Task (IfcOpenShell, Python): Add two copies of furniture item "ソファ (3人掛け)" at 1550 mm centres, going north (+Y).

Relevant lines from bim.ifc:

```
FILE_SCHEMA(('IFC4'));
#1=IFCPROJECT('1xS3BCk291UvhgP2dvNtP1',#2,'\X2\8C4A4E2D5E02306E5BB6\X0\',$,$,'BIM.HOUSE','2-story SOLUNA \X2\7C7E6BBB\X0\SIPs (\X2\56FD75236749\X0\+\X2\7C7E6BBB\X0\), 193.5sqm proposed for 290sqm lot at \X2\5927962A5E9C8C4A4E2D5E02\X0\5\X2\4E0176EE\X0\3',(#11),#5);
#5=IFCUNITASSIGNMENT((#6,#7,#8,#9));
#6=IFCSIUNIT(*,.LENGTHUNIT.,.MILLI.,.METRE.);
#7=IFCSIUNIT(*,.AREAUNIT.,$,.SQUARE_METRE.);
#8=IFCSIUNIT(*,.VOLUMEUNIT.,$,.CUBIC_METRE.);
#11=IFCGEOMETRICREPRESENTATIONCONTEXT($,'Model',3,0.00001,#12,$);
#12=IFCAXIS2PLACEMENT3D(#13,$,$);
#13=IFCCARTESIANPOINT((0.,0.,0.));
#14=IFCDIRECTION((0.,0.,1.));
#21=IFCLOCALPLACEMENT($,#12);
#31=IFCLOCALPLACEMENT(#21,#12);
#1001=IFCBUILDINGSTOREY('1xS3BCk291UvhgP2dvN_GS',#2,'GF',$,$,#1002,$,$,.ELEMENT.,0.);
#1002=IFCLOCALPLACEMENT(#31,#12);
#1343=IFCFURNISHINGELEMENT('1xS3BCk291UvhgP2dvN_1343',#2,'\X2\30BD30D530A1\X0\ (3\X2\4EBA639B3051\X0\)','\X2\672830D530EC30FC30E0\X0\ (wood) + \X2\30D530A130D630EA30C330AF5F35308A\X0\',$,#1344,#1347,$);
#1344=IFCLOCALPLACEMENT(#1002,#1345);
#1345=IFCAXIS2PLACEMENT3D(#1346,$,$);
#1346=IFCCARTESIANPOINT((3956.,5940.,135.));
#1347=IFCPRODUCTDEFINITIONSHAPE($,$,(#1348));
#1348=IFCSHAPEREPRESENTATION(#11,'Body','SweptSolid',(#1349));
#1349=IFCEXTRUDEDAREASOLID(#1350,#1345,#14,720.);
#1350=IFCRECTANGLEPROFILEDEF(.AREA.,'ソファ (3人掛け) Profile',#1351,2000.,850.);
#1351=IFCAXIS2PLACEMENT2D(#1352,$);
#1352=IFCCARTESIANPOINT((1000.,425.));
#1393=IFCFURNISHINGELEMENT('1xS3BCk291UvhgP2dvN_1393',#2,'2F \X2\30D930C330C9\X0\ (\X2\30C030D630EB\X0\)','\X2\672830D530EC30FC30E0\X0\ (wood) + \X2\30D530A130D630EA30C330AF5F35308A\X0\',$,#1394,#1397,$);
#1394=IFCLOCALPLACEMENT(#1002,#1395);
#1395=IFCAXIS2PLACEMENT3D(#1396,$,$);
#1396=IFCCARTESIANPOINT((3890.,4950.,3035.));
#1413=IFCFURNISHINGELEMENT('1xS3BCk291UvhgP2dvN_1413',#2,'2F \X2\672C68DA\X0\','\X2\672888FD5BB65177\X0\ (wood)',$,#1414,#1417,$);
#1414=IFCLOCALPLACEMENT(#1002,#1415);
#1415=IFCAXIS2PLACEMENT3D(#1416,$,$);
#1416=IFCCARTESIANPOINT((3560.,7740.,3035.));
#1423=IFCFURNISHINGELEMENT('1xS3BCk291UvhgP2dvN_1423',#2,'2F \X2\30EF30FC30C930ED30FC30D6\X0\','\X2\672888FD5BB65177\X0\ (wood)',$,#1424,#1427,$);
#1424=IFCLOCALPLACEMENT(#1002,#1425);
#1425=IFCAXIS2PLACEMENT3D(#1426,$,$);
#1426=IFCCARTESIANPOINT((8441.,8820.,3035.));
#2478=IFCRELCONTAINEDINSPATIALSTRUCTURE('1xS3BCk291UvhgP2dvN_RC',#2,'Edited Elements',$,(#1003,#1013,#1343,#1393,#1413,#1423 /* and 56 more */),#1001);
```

```python
import numpy as np
import ifcopenshell
import ifcopenshell.api.geometry
import ifcopenshell.api.root
import ifcopenshell.util.element
import ifcopenshell.util.placement
import ifcopenshell.util.unit

model = ifcopenshell.open("bim.ifc")
unit_scale = ifcopenshell.util.unit.calculate_unit_scale(model)


def reuse_history(source, copy):
    """copy_class also copies each property set's owner history, people and application; keep the originals."""
    for rel in copy.IsDefinedBy:
        if rel.is_a("IfcRelDefinesByProperties") and (history := rel.RelatingPropertyDefinition.OwnerHistory):
            rel.RelatingPropertyDefinition.OwnerHistory = source.OwnerHistory
            ifcopenshell.util.element.remove_deep2(model, history)


source = model.by_guid("1xS3BCk291UvhgP2dvN_1343")
base = ifcopenshell.util.placement.get_local_placement(source.ObjectPlacement)
step = np.array([0.0, 1.0, 0.0]) * 1.55 / unit_scale

for i in range(1, 3):
    copy = ifcopenshell.api.root.copy_class(model, product=source)
    copy.Representation = ifcopenshell.util.element.copy_deep(
        model, source.Representation, exclude=["IfcGeometricRepresentationContext", "IfcRepresentationMap"]
    )
    reuse_history(source, copy)
    matrix = base.copy()
    matrix[:3, 3] += i * step
    print("added at", matrix[:3, 3].round(3) + 0.0)
    ifcopenshell.api.geometry.edit_object_placement(model, product=copy, matrix=matrix, is_si=False)

model.write("bim_v2.ifc")
```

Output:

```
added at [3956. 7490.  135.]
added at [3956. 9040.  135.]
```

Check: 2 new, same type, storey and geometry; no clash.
